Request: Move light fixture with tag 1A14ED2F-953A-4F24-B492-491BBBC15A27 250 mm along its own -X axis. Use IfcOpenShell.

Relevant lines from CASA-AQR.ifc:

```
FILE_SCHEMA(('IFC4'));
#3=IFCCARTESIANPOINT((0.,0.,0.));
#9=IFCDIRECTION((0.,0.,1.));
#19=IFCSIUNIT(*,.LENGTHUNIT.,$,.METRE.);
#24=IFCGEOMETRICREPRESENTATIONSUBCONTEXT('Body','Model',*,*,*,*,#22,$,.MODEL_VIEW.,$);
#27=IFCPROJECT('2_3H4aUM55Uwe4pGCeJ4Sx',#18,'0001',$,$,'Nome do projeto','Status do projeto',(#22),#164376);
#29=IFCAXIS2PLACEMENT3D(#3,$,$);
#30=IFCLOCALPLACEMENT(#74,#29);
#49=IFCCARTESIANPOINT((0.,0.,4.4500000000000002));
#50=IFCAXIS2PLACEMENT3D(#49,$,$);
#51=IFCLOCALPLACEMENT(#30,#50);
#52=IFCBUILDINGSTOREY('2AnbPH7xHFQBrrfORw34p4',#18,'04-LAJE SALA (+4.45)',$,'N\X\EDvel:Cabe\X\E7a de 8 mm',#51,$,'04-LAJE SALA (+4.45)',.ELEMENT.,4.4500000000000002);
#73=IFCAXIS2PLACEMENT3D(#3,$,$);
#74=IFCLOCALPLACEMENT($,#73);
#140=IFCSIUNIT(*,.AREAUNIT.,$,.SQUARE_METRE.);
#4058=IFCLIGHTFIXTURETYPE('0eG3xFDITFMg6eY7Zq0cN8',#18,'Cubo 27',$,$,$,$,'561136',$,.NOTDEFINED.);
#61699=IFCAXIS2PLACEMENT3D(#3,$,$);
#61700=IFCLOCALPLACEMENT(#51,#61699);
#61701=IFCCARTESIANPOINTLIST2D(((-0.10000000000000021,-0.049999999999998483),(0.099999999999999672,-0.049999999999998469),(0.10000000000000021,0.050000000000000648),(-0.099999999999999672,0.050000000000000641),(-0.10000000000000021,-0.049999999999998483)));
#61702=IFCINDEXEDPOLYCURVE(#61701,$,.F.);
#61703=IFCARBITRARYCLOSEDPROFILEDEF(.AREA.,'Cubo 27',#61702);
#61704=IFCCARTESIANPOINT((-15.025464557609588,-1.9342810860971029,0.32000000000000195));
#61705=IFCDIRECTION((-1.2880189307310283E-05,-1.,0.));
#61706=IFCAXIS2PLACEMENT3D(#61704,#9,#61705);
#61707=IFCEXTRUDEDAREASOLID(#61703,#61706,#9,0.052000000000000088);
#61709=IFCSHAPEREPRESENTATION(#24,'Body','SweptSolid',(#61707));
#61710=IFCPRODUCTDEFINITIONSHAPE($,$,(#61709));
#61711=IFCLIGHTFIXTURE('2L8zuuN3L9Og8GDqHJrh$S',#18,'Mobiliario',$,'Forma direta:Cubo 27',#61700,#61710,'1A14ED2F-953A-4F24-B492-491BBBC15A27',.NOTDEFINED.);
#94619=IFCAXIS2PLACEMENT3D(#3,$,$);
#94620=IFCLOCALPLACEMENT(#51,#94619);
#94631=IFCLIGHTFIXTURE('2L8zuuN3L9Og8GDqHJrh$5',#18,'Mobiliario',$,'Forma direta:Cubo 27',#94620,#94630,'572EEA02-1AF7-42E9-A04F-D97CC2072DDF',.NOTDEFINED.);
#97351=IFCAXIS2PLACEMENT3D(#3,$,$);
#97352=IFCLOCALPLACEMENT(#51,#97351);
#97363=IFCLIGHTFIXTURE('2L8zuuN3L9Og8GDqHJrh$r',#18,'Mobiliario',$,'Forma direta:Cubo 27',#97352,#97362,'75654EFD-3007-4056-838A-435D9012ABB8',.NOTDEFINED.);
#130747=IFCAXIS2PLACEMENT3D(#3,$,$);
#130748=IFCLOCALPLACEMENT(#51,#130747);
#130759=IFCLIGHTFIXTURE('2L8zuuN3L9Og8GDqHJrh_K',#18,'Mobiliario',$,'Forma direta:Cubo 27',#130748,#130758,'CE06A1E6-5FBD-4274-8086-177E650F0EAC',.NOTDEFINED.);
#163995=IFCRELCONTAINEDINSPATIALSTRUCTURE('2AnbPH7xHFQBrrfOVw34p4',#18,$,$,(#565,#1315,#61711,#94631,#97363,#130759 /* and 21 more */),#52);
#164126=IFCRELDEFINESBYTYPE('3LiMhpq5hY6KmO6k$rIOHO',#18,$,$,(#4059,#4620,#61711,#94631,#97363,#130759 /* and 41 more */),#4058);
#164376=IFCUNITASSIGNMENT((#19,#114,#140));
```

```python
import ifcopenshell
import ifcopenshell.api.geometry
import ifcopenshell.util.placement

model = ifcopenshell.open("CASA-AQR.ifc")

item = model.by_guid("2L8zuuN3L9Og8GDqHJrh$S")
matrix = ifcopenshell.util.placement.get_local_placement(item.ObjectPlacement)
matrix[:3, 3] -= matrix[:3, 0] * 0.25
ifcopenshell.api.geometry.edit_object_placement(model, product=item, matrix=matrix, is_si=False)

print(ifcopenshell.util.placement.get_local_placement(item.ObjectPlacement).round(3) + 0.0)

model.write("CASA-AQR_updated.ifc")
```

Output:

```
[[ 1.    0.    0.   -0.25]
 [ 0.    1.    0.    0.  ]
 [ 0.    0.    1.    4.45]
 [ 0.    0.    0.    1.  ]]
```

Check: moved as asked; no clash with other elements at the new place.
